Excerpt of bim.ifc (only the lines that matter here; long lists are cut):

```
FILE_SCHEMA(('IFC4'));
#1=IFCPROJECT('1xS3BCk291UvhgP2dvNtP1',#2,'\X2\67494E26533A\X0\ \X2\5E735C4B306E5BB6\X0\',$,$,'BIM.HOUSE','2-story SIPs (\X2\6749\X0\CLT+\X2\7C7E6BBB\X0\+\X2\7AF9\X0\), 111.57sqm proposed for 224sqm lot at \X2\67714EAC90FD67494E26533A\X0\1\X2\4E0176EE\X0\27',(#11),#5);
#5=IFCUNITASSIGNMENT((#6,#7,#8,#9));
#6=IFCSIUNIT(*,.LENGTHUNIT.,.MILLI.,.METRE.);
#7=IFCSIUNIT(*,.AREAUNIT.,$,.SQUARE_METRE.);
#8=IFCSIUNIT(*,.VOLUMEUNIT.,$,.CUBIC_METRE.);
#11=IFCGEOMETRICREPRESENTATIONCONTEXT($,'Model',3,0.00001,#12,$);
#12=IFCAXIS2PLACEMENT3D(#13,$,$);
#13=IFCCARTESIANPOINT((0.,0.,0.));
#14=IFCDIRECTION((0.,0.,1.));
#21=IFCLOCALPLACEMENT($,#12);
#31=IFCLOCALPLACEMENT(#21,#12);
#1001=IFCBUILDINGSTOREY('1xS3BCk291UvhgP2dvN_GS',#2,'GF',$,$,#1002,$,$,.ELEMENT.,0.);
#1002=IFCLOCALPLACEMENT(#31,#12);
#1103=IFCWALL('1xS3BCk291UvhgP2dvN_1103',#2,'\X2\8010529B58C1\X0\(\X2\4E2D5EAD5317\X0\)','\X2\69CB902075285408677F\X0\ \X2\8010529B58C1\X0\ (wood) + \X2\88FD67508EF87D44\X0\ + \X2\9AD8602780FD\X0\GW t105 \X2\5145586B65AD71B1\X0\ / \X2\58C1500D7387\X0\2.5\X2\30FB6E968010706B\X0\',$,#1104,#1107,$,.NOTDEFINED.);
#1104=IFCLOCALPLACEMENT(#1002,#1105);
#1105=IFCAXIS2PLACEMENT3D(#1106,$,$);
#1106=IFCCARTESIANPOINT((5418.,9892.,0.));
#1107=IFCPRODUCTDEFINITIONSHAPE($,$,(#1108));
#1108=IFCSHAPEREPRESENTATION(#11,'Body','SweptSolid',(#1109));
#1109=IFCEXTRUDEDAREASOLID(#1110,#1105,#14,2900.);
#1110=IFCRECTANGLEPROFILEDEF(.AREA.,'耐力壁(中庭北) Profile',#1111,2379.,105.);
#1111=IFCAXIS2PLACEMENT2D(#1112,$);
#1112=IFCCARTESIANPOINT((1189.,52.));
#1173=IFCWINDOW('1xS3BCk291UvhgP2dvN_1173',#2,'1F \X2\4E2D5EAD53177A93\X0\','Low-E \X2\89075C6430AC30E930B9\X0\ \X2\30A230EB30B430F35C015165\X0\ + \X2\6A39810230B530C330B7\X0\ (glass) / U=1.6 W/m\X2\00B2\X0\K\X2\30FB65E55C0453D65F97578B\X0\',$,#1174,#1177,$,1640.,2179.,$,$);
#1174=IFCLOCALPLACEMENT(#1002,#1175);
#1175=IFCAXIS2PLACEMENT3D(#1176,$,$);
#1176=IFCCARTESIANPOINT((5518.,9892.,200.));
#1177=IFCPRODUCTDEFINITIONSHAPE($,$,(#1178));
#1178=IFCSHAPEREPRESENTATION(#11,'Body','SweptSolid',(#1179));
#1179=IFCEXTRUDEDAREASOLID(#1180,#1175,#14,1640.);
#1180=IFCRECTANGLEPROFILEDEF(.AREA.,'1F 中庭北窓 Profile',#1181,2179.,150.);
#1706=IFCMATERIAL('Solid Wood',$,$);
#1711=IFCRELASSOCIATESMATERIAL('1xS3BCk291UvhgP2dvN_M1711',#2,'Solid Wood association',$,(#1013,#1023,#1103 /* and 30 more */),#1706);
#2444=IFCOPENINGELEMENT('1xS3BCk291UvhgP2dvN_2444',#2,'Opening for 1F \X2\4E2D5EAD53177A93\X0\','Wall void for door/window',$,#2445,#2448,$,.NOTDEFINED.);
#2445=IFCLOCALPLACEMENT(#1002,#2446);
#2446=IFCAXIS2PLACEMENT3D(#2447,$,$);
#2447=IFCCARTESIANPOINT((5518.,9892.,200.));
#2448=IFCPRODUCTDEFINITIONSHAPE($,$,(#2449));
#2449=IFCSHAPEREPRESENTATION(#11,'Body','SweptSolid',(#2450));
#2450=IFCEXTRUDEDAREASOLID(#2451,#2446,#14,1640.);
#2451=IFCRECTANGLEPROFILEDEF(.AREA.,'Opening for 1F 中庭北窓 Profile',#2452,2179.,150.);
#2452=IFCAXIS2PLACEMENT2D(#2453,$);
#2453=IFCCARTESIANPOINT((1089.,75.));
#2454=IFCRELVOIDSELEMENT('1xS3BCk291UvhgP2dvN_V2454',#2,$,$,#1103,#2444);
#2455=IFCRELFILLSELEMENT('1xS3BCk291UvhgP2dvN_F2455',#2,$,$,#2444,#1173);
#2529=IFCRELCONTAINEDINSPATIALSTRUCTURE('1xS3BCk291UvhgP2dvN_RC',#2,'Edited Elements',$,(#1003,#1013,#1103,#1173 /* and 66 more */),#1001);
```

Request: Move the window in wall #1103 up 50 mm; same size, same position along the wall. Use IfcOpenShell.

```python
import numpy as np
import ifcopenshell
import ifcopenshell.api.geometry
import ifcopenshell.util.placement
import ifcopenshell.util.unit

model = ifcopenshell.open("bim.ifc")
unit_scale = ifcopenshell.util.unit.calculate_unit_scale(model)

window = model.by_guid("1xS3BCk291UvhgP2dvN_1173")
opening = window.FillsVoids[0].RelatingOpeningElement
dz = 50.0

shift = np.array([0.0, 0.0, dz])
# The window is not placed relative to its opening, so move both.
for product in (opening, window):
    matrix = ifcopenshell.util.placement.get_local_placement(product.ObjectPlacement)
    matrix[:3, 3] += shift
    ifcopenshell.api.geometry.edit_object_placement(model, product=product, matrix=matrix, is_si=False)

print(f"moved by {dz * unit_scale:+.3f} m")

model.write("bim_edited.ifc")
```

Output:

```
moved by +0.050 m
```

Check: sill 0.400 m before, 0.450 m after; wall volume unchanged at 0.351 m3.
